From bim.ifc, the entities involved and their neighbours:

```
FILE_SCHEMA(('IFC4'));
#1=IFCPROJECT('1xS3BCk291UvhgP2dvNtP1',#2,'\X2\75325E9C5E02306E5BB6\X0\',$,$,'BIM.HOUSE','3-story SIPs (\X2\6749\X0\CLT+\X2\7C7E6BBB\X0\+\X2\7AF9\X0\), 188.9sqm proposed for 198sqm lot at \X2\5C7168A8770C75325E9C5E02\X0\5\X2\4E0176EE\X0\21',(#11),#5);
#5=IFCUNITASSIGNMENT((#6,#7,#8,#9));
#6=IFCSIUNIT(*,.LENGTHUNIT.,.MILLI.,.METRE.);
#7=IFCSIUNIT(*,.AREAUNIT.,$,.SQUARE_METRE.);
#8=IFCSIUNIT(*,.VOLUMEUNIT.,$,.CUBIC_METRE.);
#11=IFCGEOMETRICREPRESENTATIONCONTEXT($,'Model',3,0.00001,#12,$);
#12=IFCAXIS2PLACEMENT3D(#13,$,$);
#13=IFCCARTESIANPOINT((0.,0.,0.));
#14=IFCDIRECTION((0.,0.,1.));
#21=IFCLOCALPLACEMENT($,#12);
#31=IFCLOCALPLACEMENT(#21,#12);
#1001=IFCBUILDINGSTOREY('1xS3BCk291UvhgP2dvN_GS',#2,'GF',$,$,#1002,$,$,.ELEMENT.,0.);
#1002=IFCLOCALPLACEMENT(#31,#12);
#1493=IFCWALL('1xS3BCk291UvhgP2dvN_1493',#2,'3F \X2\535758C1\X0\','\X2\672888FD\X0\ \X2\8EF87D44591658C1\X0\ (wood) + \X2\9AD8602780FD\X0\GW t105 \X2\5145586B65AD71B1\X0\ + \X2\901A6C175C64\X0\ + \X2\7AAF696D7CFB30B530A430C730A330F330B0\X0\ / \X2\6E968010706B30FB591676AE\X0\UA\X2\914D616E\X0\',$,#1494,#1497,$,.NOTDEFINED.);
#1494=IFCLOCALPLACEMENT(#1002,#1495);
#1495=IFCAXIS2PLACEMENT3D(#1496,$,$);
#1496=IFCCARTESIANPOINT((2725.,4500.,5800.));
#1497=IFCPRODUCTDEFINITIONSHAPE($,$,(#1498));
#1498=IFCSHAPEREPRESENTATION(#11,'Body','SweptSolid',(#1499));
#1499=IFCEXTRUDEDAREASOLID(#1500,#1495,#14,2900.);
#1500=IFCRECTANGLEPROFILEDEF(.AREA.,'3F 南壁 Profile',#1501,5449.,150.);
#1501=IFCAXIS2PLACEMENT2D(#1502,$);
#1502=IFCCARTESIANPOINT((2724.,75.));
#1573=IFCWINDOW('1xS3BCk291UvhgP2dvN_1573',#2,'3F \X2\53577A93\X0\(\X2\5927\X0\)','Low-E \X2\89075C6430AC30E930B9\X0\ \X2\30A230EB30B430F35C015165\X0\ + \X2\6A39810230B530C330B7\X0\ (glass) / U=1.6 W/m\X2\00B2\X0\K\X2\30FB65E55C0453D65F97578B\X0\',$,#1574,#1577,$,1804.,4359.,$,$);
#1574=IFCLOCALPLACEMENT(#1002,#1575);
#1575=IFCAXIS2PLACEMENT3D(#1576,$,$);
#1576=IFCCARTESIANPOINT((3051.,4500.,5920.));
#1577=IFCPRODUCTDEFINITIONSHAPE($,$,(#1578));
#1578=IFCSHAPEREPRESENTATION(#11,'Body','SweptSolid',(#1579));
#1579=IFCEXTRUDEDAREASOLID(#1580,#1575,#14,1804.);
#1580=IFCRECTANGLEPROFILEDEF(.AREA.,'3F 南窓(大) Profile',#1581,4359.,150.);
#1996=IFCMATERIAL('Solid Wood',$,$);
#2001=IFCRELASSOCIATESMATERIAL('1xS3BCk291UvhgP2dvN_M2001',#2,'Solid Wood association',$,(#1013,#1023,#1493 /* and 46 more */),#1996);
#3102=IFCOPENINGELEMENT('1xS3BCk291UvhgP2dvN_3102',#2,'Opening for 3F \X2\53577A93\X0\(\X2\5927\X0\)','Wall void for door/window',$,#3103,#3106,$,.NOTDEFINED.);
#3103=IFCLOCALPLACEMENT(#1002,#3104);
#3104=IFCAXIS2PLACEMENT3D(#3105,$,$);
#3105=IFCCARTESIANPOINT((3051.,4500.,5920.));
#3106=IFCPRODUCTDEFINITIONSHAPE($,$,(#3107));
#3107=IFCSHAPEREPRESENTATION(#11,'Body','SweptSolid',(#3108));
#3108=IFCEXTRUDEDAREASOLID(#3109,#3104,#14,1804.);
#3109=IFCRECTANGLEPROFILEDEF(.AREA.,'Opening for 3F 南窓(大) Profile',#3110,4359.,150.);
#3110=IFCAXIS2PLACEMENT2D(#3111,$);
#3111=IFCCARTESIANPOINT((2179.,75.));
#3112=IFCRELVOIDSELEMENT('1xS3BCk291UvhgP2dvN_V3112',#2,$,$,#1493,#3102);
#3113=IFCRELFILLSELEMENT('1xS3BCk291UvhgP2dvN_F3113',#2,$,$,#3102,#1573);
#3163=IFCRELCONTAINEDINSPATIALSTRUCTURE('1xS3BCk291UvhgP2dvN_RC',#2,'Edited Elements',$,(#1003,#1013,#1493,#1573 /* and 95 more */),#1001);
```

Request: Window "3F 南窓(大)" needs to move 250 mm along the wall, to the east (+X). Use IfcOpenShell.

```python
import ifcopenshell
import ifcopenshell.api.geometry
import ifcopenshell.util.placement

model = ifcopenshell.open("bim.ifc")

window = model.by_guid("1xS3BCk291UvhgP2dvN_1573")
opening = window.FillsVoids[0].RelatingOpeningElement
wall = opening.VoidsElements[0].RelatingBuildingElement

wall_matrix = ifcopenshell.util.placement.get_local_placement(wall.ObjectPlacement)
shift = wall_matrix[:3, 0] * 250.0
before = ifcopenshell.util.placement.get_local_placement(window.ObjectPlacement)[:3, 3].copy()

# The window is not placed relative to its opening, so move both.
for product in (opening, window):
    matrix = ifcopenshell.util.placement.get_local_placement(product.ObjectPlacement)
    matrix[:3, 3] += shift
    ifcopenshell.api.geometry.edit_object_placement(model, product=product, matrix=matrix, is_si=False)

after = ifcopenshell.util.placement.get_local_placement(window.ObjectPlacement)[:3, 3]
print("window moved by", (after - before).round(3) + 0.0)

model.write("bim_v2.ifc")
```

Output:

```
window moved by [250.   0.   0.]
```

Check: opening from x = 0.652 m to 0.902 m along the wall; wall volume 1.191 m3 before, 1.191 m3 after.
